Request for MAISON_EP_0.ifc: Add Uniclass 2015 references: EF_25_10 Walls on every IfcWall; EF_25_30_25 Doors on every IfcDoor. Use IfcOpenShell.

First a look at what the model holds.

```python
import ifcopenshell

model = ifcopenshell.open("MAISON_EP_0.ifc")
print(model.schema)
print("classifications:", [c.Name for c in model.by_type("IfcClassification")])
for ifc_class in ("IfcDoor", "IfcRoof", "IfcStair", "IfcWall", "IfcWindow"):
    print(ifc_class, len(model.by_type(ifc_class)))
```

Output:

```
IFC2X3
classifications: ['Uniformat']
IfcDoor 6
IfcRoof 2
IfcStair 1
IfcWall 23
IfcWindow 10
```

```python
import ifcopenshell
import ifcopenshell.api.classification

model = ifcopenshell.open("MAISON_EP_0.ifc")

# IFC2X3 requires Source and Edition and has no link from the project to the system.
system = model.create_entity("IfcClassification", Source="NBS", Edition="2015", Name="Uniclass 2015")

codes = {
    "IfcWall": ("EF_25_10", "Walls"),
    "IfcDoor": ("EF_25_30_25", "Doors"),
}
for ifc_class, (code, name) in codes.items():
    products = model.by_type(ifc_class)
    ifcopenshell.api.classification.add_reference(
        model, products=products, classification=system, identification=code, name=name
    )
    print(code, len(products))

model.write("MAISON_EP_0-out.ifc")
```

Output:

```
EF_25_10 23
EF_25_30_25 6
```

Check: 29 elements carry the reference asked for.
